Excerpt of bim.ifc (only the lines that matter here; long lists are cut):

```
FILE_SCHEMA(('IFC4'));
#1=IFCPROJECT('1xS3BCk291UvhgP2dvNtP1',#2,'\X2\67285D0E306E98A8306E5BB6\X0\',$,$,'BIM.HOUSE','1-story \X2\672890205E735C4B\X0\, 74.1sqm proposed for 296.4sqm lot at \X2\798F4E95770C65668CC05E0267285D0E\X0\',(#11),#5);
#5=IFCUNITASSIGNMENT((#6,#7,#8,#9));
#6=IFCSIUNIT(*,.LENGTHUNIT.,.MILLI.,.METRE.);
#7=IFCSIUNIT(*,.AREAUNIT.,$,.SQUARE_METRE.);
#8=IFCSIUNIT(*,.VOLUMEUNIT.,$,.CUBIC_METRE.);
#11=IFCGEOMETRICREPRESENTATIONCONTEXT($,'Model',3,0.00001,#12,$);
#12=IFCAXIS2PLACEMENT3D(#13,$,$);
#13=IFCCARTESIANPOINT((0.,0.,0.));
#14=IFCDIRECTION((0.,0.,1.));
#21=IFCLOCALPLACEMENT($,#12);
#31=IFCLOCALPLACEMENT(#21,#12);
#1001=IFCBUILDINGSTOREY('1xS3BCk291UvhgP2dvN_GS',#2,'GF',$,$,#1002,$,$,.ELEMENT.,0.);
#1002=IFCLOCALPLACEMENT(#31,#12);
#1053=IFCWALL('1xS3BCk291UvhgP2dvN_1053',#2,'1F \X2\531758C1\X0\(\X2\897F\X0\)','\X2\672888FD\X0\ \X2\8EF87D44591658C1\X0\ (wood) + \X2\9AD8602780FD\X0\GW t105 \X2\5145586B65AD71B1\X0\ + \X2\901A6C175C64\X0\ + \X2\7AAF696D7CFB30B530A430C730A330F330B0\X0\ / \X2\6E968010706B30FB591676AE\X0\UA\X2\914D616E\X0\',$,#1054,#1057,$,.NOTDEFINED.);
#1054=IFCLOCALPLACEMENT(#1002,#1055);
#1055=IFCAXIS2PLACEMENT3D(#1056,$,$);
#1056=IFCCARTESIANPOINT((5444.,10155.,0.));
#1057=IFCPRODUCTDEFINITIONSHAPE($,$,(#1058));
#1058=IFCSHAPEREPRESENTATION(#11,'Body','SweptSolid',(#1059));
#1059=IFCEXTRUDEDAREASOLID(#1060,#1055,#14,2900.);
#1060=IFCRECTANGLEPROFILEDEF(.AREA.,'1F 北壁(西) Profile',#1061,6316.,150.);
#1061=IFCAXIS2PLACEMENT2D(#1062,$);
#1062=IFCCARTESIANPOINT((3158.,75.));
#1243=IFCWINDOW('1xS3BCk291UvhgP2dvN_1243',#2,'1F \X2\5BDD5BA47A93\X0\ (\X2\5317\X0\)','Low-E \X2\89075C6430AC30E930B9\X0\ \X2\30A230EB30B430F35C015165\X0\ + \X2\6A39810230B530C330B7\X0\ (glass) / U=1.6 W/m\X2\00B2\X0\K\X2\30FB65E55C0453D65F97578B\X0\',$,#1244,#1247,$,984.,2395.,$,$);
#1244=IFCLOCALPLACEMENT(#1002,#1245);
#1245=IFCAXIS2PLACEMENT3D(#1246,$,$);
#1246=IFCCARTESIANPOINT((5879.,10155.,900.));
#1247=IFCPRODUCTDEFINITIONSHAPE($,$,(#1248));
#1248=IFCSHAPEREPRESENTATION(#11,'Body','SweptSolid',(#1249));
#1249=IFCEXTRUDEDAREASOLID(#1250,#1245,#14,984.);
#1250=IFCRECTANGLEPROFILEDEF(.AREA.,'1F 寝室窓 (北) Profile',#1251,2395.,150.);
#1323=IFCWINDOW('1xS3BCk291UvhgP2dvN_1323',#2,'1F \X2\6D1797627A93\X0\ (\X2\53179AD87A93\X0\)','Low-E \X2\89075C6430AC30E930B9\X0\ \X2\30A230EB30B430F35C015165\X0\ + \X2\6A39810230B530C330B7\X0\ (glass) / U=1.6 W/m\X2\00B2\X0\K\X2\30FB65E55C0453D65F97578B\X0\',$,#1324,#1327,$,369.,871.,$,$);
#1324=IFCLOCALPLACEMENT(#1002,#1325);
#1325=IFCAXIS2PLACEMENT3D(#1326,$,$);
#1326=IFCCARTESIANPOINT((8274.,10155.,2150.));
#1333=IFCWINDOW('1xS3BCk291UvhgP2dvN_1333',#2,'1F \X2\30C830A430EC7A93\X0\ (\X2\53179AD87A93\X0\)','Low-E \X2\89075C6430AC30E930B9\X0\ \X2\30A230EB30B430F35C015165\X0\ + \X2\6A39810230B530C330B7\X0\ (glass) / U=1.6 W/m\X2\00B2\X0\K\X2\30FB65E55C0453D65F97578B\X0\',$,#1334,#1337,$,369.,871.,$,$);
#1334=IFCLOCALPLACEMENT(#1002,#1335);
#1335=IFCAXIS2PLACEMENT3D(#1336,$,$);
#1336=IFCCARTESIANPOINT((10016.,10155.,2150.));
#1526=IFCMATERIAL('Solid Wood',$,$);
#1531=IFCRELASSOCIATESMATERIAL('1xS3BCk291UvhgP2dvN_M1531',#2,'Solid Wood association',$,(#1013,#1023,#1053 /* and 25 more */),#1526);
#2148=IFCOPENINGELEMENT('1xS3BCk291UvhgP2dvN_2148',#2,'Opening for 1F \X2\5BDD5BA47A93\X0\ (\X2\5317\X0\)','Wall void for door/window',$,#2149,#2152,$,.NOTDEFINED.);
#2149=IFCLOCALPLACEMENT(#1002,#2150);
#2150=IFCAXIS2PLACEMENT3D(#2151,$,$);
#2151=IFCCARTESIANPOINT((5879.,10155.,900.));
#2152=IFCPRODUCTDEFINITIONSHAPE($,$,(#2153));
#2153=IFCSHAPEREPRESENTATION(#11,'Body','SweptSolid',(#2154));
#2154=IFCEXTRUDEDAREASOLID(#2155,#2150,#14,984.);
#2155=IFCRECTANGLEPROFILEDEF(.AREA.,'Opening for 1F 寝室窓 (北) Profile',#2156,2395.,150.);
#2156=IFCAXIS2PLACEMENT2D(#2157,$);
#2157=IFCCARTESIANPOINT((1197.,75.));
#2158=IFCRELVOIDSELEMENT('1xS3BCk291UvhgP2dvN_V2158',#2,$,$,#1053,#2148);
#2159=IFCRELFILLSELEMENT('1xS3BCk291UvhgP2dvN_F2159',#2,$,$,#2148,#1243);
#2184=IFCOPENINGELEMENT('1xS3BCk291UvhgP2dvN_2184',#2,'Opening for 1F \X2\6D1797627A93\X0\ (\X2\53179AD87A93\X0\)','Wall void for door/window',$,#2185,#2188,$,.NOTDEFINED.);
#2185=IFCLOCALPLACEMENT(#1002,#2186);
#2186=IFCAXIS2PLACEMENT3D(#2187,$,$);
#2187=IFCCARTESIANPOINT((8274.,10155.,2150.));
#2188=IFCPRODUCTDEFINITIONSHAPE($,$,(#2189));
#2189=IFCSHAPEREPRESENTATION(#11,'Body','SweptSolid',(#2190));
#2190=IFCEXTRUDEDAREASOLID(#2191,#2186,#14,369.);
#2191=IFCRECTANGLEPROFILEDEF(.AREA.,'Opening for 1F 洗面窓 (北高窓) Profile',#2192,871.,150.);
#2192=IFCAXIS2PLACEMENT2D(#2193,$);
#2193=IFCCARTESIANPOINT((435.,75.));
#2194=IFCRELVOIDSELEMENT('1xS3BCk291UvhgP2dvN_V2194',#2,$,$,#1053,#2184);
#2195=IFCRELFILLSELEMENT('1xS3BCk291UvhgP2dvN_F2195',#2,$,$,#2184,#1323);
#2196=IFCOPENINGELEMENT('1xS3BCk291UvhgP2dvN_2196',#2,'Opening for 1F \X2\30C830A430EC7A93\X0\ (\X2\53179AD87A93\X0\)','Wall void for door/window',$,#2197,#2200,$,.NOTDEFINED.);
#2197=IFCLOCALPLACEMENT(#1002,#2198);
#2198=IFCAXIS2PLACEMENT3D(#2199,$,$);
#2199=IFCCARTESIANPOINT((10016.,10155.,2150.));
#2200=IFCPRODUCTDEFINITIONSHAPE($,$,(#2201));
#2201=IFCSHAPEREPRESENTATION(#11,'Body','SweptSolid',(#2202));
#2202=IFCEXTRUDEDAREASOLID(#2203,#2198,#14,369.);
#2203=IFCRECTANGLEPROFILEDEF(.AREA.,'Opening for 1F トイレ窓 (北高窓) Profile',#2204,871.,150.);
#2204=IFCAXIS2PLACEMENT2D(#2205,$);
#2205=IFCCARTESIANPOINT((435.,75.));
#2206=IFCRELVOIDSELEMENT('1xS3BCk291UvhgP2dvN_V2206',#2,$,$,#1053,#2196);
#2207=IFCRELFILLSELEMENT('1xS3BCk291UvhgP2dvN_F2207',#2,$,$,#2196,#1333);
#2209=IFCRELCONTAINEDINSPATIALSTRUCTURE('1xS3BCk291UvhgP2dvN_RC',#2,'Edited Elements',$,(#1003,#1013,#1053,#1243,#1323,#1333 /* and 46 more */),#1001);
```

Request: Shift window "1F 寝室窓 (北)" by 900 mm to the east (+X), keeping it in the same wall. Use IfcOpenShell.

```python
import ifcopenshell
import ifcopenshell.api.geometry
import ifcopenshell.util.placement
import ifcopenshell.util.unit

model = ifcopenshell.open("bim.ifc")
unit_scale = ifcopenshell.util.unit.calculate_unit_scale(model)

window = model.by_guid("1xS3BCk291UvhgP2dvN_1243")
opening = window.FillsVoids[0].RelatingOpeningElement
wall = opening.VoidsElements[0].RelatingBuildingElement

wall_matrix = ifcopenshell.util.placement.get_local_placement(wall.ObjectPlacement)
shift = wall_matrix[:3, 0] * 0.9 / unit_scale
before = ifcopenshell.util.placement.get_local_placement(window.ObjectPlacement)[:3, 3].copy()

# The window is not placed relative to its opening, so move both.
for product in (opening, window):
    matrix = ifcopenshell.util.placement.get_local_placement(product.ObjectPlacement)
    matrix[:3, 3] += shift
    ifcopenshell.api.geometry.edit_object_placement(model, product=product, matrix=matrix, is_si=False)

after = ifcopenshell.util.placement.get_local_placement(window.ObjectPlacement)[:3, 3]
print("window moved by", (after - before).round(3) + 0.0)

model.write("bim_updated.ifc")
```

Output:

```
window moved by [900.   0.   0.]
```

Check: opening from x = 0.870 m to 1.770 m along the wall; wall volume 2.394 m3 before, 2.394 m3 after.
